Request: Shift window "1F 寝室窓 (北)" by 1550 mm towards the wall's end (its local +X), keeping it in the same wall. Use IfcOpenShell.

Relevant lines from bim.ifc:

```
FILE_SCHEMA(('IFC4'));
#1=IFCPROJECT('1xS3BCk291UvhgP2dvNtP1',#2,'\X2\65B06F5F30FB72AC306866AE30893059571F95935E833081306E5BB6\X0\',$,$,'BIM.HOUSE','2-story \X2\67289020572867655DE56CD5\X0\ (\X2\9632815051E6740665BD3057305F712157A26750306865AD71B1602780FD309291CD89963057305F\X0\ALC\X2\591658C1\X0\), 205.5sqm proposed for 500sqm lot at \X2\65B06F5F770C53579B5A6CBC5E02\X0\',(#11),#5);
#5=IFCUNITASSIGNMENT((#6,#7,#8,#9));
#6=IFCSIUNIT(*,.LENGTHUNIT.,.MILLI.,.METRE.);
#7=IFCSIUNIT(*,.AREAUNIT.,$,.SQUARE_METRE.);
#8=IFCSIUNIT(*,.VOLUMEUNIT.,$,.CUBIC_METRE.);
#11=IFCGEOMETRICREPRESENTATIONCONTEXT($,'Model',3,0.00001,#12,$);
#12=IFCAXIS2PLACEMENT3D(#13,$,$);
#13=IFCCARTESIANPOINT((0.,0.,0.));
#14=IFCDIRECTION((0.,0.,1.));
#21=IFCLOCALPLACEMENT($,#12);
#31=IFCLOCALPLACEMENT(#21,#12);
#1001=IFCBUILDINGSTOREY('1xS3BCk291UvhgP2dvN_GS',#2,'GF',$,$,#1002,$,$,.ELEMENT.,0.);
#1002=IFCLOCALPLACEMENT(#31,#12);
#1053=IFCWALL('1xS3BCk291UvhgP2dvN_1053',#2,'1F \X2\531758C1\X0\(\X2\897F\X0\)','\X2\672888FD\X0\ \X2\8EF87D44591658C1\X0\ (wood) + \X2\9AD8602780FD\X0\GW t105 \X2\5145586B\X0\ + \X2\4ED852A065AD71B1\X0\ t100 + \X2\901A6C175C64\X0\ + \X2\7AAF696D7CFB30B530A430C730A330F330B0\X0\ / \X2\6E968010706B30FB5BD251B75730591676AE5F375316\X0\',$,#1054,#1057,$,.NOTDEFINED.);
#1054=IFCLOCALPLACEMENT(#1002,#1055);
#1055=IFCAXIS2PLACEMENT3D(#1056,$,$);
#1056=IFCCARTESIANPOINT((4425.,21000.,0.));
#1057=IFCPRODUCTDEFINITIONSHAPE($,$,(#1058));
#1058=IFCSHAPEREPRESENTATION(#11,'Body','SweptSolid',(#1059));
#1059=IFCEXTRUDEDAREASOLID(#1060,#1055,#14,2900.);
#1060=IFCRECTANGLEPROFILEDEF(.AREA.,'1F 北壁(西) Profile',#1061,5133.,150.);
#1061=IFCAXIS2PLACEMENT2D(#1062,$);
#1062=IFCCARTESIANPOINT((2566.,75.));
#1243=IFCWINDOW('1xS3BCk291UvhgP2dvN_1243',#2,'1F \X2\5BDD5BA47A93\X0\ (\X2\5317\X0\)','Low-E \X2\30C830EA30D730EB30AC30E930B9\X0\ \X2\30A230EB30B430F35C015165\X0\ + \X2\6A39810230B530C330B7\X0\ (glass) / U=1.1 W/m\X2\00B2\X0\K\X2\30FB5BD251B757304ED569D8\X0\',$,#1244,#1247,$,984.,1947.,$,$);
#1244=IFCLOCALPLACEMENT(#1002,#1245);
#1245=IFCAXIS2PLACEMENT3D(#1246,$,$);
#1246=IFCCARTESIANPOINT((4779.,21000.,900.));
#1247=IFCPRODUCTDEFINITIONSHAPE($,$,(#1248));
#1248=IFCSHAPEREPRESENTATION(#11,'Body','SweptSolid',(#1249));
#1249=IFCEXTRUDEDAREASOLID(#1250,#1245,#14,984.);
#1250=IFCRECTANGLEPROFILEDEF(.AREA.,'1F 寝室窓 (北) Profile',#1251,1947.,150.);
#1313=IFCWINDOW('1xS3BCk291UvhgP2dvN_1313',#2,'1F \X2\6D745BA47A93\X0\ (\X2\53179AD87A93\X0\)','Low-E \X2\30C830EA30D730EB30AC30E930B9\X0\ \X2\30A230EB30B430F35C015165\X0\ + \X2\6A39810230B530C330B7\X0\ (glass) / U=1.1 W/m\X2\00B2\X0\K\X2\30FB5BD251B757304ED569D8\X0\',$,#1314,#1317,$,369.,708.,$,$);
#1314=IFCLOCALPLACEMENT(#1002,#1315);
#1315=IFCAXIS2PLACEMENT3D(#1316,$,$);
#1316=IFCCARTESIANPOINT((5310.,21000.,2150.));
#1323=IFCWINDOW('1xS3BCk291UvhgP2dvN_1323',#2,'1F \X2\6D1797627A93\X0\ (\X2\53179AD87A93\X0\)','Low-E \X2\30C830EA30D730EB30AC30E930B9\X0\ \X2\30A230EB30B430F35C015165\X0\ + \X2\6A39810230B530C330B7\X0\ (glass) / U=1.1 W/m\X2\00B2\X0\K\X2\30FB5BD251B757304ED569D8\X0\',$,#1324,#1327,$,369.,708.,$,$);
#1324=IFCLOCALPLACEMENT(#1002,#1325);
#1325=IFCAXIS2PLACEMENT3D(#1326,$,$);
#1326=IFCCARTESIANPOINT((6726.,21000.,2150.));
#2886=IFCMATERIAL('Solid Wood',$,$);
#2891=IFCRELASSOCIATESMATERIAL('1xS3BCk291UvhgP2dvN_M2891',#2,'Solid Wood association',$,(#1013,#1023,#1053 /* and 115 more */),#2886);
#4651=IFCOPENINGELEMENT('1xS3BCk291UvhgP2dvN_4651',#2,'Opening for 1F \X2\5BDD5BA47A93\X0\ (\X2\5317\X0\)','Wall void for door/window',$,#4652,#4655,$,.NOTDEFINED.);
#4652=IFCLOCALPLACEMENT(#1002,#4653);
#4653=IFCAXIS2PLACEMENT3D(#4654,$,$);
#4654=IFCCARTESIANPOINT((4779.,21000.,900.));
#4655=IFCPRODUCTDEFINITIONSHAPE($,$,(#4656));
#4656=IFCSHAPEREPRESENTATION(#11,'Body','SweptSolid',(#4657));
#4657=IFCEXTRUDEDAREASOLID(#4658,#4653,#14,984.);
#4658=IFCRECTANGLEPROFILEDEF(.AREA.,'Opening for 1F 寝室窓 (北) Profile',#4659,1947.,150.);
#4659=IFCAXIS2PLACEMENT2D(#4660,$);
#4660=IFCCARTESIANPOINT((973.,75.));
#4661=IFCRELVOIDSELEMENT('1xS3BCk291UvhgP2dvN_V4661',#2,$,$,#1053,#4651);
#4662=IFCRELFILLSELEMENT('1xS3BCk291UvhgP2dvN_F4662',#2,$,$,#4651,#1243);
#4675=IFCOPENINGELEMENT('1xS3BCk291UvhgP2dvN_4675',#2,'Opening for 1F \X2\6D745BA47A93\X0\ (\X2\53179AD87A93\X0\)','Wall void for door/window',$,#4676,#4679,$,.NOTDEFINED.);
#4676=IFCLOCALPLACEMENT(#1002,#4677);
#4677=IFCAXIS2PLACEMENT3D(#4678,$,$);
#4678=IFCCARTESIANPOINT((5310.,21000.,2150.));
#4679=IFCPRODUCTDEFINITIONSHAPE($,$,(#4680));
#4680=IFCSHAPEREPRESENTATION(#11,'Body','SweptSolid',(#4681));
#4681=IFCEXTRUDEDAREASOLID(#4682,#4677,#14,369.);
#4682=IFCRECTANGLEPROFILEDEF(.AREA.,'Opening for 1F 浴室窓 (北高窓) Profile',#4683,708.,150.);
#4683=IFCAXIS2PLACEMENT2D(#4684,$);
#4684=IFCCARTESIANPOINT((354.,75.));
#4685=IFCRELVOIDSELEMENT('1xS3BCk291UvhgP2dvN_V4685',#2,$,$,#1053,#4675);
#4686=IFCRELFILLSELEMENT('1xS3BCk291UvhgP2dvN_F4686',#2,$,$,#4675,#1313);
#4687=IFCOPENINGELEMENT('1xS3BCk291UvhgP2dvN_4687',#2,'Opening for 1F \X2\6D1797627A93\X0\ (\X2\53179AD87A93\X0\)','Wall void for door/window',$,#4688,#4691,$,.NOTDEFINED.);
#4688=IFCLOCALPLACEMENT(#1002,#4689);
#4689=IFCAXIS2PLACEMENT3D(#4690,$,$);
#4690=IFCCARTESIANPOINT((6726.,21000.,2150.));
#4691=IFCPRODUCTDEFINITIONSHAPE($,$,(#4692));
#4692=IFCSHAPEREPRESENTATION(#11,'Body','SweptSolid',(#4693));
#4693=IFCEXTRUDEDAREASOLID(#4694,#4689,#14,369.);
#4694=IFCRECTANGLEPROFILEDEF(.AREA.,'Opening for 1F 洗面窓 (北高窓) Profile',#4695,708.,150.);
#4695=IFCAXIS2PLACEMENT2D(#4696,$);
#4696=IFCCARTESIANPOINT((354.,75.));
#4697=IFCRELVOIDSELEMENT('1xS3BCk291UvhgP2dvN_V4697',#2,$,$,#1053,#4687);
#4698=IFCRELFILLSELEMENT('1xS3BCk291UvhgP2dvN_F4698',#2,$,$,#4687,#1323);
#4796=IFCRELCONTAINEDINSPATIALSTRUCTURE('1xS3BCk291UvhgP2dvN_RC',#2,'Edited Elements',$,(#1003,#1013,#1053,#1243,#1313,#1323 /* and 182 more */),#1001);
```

```python
import ifcopenshell
import ifcopenshell.api.geometry
import ifcopenshell.util.placement

model = ifcopenshell.open("bim.ifc")

window = model.by_guid("1xS3BCk291UvhgP2dvN_1243")
opening = window.FillsVoids[0].RelatingOpeningElement
wall = opening.VoidsElements[0].RelatingBuildingElement

wall_matrix = ifcopenshell.util.placement.get_local_placement(wall.ObjectPlacement)
shift = wall_matrix[:3, 0] * 1550.0
before = ifcopenshell.util.placement.get_local_placement(window.ObjectPlacement)[:3, 3].copy()

# The window is not placed relative to its opening, so move both.
for product in (opening, window):
    matrix = ifcopenshell.util.placement.get_local_placement(product.ObjectPlacement)
    matrix[:3, 3] += shift
    ifcopenshell.api.geometry.edit_object_placement(model, product=product, matrix=matrix, is_si=False)

after = ifcopenshell.util.placement.get_local_placement(window.ObjectPlacement)[:3, 3]
print("window moved by", (after - before).round(3) + 0.0)

model.write("bim_rev.ifc")
```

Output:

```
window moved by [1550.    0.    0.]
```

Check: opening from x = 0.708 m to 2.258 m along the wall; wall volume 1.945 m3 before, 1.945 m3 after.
